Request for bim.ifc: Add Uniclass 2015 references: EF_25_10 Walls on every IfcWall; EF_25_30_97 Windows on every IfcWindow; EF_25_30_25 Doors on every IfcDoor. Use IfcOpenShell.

First a look at what the model holds.

```python
import ifcopenshell

model = ifcopenshell.open("bim.ifc")
print(model.schema)
print("classifications:", [c.Name for c in model.by_type("IfcClassification")])
for ifc_class in ("IfcDoor", "IfcRoof", "IfcStair", "IfcWall", "IfcWindow"):
    print(ifc_class, len(model.by_type(ifc_class)))
```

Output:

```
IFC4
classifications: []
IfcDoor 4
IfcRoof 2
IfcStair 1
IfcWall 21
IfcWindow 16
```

```python
import ifcopenshell
import ifcopenshell.api.classification

model = ifcopenshell.open("bim.ifc")

system = ifcopenshell.api.classification.add_classification(model, classification="Uniclass 2015")

codes = {
    "IfcWall": ("EF_25_10", "Walls"),
    "IfcWindow": ("EF_25_30_97", "Windows"),
    "IfcDoor": ("EF_25_30_25", "Doors"),
}
for ifc_class, (code, name) in codes.items():
    products = model.by_type(ifc_class)
    ifcopenshell.api.classification.add_reference(
        model, products=products, classification=system, identification=code, name=name
    )
    print(code, len(products))

model.write("bim_edited.ifc")
```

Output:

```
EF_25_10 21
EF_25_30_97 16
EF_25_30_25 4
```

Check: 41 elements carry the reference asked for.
